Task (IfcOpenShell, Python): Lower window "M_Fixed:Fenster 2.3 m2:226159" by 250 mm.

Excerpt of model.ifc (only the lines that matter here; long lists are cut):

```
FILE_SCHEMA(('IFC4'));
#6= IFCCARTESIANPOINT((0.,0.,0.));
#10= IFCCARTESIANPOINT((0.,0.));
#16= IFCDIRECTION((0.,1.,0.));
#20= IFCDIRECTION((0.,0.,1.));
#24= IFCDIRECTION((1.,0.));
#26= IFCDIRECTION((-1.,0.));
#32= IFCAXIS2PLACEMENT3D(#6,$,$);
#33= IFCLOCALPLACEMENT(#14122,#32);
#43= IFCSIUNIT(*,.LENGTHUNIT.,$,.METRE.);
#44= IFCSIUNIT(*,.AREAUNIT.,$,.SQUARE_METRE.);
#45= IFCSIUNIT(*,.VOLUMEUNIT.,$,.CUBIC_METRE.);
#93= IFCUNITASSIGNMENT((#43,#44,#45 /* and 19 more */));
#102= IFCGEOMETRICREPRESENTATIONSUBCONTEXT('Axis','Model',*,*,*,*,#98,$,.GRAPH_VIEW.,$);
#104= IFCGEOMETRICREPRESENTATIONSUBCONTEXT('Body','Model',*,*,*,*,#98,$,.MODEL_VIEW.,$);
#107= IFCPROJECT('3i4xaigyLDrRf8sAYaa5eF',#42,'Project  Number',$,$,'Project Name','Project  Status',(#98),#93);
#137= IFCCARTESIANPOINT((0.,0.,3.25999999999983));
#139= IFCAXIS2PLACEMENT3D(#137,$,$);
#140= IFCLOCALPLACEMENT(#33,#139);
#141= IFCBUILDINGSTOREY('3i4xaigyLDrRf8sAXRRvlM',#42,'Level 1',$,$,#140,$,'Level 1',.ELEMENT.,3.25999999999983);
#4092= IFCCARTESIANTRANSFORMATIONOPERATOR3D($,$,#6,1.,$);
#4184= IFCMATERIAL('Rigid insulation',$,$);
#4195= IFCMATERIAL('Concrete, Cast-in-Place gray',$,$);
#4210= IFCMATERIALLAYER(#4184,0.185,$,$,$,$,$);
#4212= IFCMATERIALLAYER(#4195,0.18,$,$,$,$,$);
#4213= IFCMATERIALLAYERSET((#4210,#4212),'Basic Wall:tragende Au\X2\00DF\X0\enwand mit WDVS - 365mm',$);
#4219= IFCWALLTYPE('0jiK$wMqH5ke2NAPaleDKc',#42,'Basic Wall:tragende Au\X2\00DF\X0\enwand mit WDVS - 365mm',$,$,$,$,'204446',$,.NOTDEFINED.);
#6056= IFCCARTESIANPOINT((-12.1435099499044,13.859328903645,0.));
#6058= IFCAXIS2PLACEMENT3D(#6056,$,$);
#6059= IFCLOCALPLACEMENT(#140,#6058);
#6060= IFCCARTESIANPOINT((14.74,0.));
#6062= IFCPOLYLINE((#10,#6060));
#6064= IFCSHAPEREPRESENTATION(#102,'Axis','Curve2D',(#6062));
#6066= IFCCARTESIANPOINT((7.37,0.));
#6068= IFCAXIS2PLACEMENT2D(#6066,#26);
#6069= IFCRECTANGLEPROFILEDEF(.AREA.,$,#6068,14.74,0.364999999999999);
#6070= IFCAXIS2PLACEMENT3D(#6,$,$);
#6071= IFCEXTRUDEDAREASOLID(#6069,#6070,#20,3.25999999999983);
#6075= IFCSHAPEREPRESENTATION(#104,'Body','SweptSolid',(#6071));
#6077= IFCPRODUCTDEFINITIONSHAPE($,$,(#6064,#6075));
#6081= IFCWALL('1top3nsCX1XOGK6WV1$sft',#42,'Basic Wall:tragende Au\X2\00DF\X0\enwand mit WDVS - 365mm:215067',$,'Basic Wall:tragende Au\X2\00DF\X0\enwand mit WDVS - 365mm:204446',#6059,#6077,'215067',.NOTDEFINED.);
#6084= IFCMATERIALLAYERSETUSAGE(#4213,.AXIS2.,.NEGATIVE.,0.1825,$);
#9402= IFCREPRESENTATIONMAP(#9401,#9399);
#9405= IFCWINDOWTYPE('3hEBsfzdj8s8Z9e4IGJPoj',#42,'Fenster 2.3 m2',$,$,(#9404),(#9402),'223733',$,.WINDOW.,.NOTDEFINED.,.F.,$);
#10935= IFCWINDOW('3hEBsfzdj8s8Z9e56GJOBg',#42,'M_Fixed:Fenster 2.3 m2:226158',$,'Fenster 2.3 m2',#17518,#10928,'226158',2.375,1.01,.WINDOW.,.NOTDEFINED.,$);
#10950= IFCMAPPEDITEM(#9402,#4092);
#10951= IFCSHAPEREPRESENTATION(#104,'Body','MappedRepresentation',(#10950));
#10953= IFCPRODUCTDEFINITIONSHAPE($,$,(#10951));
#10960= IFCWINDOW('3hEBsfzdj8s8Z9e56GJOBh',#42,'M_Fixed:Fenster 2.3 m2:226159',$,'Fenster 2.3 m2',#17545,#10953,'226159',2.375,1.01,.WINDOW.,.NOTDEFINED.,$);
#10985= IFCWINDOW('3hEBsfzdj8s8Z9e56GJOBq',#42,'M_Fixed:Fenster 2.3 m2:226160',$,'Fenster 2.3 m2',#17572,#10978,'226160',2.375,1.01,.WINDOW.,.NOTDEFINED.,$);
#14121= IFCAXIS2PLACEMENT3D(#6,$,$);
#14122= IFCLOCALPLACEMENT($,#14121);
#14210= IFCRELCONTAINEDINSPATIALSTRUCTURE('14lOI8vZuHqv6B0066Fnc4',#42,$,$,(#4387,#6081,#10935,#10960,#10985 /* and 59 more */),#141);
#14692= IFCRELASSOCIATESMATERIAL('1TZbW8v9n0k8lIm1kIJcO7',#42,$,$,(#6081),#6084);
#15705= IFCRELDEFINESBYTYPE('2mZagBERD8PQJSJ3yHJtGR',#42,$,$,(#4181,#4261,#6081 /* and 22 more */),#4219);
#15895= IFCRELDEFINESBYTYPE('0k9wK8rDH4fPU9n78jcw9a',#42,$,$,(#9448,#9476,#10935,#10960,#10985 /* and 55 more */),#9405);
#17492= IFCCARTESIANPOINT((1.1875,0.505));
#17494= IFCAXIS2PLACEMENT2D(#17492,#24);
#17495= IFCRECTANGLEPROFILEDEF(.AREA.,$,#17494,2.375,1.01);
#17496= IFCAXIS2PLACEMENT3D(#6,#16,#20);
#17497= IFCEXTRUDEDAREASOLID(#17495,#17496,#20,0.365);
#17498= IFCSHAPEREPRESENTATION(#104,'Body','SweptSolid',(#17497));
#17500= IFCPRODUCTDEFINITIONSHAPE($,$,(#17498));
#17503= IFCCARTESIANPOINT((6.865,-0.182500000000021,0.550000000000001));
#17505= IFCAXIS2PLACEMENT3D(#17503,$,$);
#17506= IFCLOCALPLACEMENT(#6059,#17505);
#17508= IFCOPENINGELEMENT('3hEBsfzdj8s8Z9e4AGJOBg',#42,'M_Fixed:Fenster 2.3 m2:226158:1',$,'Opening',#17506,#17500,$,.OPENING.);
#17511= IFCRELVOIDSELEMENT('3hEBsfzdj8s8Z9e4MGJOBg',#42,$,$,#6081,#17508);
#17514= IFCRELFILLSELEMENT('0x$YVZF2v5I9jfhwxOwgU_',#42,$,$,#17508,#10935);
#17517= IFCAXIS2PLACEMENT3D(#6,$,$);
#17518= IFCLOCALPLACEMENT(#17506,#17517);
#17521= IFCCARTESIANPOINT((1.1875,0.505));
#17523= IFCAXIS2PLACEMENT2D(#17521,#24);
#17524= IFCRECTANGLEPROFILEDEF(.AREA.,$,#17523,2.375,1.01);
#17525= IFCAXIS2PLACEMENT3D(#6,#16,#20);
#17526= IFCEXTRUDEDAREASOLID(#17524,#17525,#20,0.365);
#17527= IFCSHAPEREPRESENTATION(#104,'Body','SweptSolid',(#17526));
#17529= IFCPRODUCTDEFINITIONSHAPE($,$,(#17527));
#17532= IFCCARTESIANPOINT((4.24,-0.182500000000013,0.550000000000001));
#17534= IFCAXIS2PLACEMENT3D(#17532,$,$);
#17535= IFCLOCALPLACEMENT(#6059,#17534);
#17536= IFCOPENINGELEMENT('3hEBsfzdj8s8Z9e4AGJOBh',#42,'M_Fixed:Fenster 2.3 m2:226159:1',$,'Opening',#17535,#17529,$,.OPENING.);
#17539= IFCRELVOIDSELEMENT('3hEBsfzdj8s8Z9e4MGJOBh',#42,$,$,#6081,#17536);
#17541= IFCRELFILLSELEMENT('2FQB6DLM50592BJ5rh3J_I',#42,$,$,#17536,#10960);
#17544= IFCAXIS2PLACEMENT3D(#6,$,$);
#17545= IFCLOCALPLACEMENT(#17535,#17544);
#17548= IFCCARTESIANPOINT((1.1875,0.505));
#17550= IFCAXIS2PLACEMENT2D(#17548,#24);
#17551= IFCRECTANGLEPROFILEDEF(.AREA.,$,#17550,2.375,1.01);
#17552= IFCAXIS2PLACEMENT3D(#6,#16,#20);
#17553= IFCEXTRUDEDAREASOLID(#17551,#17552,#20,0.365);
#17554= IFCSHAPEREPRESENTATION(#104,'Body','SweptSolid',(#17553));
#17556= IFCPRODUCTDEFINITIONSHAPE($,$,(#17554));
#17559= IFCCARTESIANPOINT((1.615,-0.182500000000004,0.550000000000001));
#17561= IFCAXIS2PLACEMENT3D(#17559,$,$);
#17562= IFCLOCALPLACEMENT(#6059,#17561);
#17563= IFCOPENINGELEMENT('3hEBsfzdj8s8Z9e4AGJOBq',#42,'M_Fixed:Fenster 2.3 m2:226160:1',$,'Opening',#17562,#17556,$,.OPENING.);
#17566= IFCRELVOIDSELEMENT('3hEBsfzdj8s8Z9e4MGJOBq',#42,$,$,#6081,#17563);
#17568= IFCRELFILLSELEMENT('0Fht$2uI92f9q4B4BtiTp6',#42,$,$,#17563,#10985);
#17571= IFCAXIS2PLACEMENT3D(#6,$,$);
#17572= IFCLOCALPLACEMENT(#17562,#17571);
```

```python
import numpy as np
import ifcopenshell
import ifcopenshell.api.geometry
import ifcopenshell.util.placement
import ifcopenshell.util.unit

model = ifcopenshell.open("model.ifc")
unit_scale = ifcopenshell.util.unit.calculate_unit_scale(model)

window = model.by_id(10960)
opening = window.FillsVoids[0].RelatingOpeningElement
dz = -0.25 / unit_scale

shift = np.array([0.0, 0.0, dz])
# The window is placed relative to its opening, so it follows when the opening moves.
matrix = ifcopenshell.util.placement.get_local_placement(opening.ObjectPlacement)
matrix[:3, 3] += shift
ifcopenshell.api.geometry.edit_object_placement(
    model, product=opening, matrix=matrix, is_si=False, should_transform_children=True
)

print(f"moved by {dz * unit_scale:+.3f} m")

model.write("model-out.ifc")
```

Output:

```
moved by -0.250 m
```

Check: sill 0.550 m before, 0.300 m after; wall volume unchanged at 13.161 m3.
